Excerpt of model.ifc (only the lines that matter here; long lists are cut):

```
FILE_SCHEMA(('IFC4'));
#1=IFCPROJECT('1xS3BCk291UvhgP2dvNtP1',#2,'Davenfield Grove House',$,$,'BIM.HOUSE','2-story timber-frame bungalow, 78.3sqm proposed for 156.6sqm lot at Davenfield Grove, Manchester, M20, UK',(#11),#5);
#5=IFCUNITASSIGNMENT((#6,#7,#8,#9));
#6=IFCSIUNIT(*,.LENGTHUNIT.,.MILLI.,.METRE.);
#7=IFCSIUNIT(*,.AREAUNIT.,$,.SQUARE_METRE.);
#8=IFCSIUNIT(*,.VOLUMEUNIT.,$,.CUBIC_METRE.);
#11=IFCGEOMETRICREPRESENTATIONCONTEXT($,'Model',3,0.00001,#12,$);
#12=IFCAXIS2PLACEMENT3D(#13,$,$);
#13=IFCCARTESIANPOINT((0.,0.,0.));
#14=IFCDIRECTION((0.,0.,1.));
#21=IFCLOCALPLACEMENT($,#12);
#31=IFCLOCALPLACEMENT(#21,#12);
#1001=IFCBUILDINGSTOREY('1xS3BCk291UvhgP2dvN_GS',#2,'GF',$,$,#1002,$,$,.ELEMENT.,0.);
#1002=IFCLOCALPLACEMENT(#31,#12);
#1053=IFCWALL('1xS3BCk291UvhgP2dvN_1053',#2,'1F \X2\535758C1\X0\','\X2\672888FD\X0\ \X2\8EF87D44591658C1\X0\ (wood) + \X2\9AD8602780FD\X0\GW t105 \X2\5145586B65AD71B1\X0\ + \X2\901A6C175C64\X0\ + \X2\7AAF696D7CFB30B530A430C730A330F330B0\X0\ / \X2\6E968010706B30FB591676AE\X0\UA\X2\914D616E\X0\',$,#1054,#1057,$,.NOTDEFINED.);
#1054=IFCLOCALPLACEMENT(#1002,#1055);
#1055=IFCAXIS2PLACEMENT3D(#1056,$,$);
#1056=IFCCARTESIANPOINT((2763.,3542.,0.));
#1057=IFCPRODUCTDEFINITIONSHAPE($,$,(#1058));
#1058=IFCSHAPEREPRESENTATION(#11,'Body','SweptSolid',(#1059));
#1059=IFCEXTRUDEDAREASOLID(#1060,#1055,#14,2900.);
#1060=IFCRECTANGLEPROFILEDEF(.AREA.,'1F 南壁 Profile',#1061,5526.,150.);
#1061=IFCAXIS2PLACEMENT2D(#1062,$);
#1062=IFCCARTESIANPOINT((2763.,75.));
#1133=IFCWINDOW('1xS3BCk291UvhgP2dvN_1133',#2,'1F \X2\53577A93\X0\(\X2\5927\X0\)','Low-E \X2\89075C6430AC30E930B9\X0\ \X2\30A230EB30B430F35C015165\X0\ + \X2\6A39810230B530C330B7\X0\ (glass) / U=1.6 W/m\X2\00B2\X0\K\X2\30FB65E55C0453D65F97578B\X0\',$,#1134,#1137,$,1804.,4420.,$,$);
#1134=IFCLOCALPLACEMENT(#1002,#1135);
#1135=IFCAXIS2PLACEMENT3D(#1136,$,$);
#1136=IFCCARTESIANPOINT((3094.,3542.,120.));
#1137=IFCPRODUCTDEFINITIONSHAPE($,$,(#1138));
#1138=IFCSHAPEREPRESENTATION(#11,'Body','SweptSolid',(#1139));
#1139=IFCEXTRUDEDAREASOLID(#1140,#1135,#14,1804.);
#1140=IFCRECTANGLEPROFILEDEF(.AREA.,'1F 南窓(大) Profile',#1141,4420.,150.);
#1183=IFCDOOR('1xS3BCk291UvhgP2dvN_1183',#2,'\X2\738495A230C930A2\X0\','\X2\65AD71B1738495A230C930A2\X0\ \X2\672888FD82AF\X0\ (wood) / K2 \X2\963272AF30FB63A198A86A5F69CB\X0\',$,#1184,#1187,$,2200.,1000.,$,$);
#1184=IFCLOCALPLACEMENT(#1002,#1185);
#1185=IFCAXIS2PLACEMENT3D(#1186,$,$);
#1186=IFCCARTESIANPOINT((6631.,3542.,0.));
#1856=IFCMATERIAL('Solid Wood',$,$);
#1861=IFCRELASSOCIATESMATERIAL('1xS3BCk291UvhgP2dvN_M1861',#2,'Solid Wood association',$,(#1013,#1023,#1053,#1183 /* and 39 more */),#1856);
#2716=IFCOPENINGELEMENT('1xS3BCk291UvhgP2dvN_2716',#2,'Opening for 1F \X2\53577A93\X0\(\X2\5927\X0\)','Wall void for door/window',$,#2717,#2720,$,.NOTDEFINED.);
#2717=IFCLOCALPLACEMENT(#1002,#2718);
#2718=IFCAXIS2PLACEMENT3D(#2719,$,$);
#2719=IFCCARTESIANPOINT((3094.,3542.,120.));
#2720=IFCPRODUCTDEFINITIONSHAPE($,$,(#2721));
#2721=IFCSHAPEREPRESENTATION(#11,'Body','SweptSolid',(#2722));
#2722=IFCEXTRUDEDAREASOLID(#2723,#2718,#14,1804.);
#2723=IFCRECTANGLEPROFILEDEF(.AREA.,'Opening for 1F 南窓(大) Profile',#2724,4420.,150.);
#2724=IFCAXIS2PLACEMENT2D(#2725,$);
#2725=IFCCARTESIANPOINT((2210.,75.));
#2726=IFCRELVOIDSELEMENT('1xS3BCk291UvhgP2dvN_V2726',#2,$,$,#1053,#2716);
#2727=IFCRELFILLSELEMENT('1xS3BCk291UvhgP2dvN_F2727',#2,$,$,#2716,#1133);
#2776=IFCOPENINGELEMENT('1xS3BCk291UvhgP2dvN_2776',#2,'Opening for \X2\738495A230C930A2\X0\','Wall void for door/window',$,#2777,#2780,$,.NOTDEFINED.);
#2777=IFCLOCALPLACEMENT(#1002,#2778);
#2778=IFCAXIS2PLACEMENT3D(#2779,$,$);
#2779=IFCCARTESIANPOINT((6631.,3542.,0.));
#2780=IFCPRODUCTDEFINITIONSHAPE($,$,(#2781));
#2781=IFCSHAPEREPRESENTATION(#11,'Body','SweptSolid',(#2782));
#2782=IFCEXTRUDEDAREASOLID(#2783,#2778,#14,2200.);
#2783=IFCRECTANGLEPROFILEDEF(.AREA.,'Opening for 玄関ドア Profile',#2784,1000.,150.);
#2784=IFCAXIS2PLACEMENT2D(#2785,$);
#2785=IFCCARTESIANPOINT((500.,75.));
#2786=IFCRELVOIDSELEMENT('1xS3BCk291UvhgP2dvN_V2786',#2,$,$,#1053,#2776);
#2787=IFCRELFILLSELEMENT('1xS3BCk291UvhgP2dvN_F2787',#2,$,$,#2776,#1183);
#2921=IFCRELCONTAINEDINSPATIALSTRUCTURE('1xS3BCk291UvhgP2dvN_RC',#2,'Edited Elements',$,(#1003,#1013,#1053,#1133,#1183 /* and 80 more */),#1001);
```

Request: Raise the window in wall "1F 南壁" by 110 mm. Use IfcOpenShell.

```python
import numpy as np
import ifcopenshell
import ifcopenshell.api.geometry
import ifcopenshell.util.placement
import ifcopenshell.util.unit

model = ifcopenshell.open("model.ifc")
unit_scale = ifcopenshell.util.unit.calculate_unit_scale(model)

window = model.by_guid("1xS3BCk291UvhgP2dvN_1133")
opening = window.FillsVoids[0].RelatingOpeningElement
dz = 0.11 / unit_scale

shift = np.array([0.0, 0.0, dz])
# The window is not placed relative to its opening, so move both.
for product in (opening, window):
    matrix = ifcopenshell.util.placement.get_local_placement(product.ObjectPlacement)
    matrix[:3, 3] += shift
    ifcopenshell.api.geometry.edit_object_placement(model, product=product, matrix=matrix, is_si=False)

print(f"moved by {dz * unit_scale:+.3f} m")

model.write("model_v2.ifc")
```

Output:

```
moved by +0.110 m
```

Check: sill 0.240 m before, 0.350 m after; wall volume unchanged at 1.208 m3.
